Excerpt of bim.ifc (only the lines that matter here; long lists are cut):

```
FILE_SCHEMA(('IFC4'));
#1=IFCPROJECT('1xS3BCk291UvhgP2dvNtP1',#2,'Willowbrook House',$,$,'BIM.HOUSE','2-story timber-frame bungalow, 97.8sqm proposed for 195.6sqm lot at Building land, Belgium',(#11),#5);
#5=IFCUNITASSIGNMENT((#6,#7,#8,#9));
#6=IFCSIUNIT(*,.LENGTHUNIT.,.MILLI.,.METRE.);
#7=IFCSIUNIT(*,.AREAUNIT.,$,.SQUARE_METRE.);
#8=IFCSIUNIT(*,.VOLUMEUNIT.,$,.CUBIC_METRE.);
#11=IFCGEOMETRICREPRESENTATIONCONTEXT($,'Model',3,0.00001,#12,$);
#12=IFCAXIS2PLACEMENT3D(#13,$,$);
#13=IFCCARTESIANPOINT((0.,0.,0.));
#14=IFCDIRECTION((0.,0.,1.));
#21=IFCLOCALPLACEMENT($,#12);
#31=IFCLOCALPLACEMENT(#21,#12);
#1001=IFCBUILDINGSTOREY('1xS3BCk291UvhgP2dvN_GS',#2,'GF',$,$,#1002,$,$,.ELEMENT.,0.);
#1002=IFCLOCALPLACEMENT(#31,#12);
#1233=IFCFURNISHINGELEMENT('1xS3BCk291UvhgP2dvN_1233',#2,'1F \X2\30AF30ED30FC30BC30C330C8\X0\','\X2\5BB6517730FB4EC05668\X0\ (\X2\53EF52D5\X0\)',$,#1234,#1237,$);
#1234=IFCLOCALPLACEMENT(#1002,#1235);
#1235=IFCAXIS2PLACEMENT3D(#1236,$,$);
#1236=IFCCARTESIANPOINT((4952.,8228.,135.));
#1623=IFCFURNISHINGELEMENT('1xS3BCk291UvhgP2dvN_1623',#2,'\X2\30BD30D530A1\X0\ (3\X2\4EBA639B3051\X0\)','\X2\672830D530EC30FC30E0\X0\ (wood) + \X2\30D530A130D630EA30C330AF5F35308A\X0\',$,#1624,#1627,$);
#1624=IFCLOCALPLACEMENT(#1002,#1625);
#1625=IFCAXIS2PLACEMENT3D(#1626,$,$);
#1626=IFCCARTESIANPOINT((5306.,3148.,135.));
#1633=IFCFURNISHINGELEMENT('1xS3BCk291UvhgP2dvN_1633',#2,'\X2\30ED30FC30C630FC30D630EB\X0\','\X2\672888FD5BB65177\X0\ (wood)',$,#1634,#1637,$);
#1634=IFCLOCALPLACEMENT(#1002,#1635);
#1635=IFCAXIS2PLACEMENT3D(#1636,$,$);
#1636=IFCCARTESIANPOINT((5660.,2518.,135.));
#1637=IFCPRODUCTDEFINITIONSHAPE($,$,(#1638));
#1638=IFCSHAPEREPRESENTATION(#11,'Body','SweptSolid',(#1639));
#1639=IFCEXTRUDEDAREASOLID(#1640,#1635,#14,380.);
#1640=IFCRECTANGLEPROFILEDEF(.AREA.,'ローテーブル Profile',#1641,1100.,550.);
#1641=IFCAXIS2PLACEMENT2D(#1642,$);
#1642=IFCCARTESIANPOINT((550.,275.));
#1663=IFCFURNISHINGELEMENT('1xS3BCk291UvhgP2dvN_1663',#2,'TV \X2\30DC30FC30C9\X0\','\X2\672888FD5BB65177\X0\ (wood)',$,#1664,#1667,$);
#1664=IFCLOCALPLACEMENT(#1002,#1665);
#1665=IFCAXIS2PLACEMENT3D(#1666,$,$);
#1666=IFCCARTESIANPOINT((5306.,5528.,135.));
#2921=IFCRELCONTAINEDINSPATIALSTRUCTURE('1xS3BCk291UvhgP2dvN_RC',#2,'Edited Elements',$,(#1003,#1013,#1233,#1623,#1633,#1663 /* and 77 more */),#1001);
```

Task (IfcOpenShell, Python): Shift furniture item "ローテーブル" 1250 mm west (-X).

```python
import ifcopenshell
import ifcopenshell.api.geometry
import ifcopenshell.util.placement

model = ifcopenshell.open("bim.ifc")

item = model.by_guid("1xS3BCk291UvhgP2dvN_1633")
matrix = ifcopenshell.util.placement.get_local_placement(item.ObjectPlacement)
matrix[0, 3] -= 1250.0
ifcopenshell.api.geometry.edit_object_placement(model, product=item, matrix=matrix, is_si=False)

print(ifcopenshell.util.placement.get_local_placement(item.ObjectPlacement).round(3) + 0.0)

model.write("bim_updated.ifc")
```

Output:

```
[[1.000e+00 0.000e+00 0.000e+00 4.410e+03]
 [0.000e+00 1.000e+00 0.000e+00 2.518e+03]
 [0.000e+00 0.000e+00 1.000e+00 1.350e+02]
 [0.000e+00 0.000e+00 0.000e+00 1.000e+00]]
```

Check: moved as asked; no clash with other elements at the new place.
